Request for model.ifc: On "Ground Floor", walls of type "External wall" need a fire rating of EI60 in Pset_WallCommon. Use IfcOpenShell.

First a look at what the model holds.

```python
import ifcopenshell
import ifcopenshell.util.element

model = ifcopenshell.open("model.ifc")
print(model.schema)
storey = next(s for s in model.by_type("IfcBuildingStorey") if s.Name == "Ground Floor")
walls = [e for e in ifcopenshell.util.element.get_decomposition(storey) if e.is_a("IfcWall")]
seen = {}
for e in walls:
    element_type = ifcopenshell.util.element.get_type(e)
    key = (element_type.Name if element_type != e and element_type else None, ifcopenshell.util.element.get_pset(e, "Pset_WallCommon", "FireRating"))
    seen[key] = seen.get(key, 0) + 1
for (name, value), count in sorted(seen.items(), key=str):
    print(count, "x", name, "|", value)
```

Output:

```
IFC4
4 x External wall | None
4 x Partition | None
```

```python
import ifcopenshell
import ifcopenshell.api.pset
import ifcopenshell.util.element

model = ifcopenshell.open("model.ifc")

storey = next(s for s in model.by_type("IfcBuildingStorey") if s.Name == "Ground Floor")
walls = [e for e in ifcopenshell.util.element.get_decomposition(storey) if e.is_a("IfcWall")]

count = 0
for e in walls:
    element_type = ifcopenshell.util.element.get_type(e)
    if element_type in (None, e) or element_type.Name != "External wall":
        continue
    # add_pset returns the element's existing set when there is one.
    pset = ifcopenshell.api.pset.add_pset(model, product=e, name="Pset_WallCommon")
    ifcopenshell.api.pset.edit_pset(model, pset=pset, properties={"FireRating": "EI60"})
    count += 1

print(count, "walls updated")

model.write("model_updated.ifc")
```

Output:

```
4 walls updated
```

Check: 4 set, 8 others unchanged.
